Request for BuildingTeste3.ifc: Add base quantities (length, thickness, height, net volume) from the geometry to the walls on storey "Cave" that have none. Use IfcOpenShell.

First a look at what the model holds.

```python
import ifcopenshell
import ifcopenshell.util.element
import ifcopenshell.util.unit

model = ifcopenshell.open("BuildingTeste3.ifc")
print(model.schema)
for unit_type in ("LENGTHUNIT", "AREAUNIT", "VOLUMEUNIT"):
    print(unit_type, ifcopenshell.util.unit.calculate_unit_scale(model, unit_type))
storey = next(s for s in model.by_type("IfcBuildingStorey") if s.Name == "Cave")
walls = [e for e in ifcopenshell.util.element.get_decomposition(storey) if e.is_a("IfcWall")]
for e in sorted(walls, key=lambda e: e.id()):
    print(e.id(), e.is_a(), e.Name, list(ifcopenshell.util.element.get_psets(e, qtos_only=True)), sep=" | ")
```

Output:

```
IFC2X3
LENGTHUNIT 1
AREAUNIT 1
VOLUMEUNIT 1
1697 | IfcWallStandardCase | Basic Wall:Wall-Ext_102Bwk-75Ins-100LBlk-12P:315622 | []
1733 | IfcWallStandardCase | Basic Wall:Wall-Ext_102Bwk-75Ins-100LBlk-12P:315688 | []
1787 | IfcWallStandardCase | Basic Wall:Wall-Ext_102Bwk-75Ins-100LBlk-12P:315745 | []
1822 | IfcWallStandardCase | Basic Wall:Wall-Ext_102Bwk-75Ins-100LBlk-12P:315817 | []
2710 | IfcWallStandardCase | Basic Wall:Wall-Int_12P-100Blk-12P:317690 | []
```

```python
import ifcopenshell
import ifcopenshell.api.pset
import ifcopenshell.geom
import ifcopenshell.util.element
import ifcopenshell.util.shape
import ifcopenshell.util.unit

model = ifcopenshell.open("BuildingTeste3.ifc")
unit_scale = ifcopenshell.util.unit.calculate_unit_scale(model)
volume_scale = ifcopenshell.util.unit.calculate_unit_scale(model, "VOLUMEUNIT")
settings = ifcopenshell.geom.settings()

storey = next(s for s in model.by_type("IfcBuildingStorey") if s.Name == "Cave")
walls = [e for e in ifcopenshell.util.element.get_decomposition(storey) if e.is_a("IfcWall")]

for e in sorted(walls, key=lambda e: e.id()):
    if ifcopenshell.util.element.get_psets(e, qtos_only=True, should_inherit=False):
        continue
    # Geometry comes back in metres, in the element's own axes.
    shape = ifcopenshell.geom.create_shape(settings, e)
    values = {
        "Length": ifcopenshell.util.shape.get_x(shape.geometry) / unit_scale,
        "Width": ifcopenshell.util.shape.get_y(shape.geometry) / unit_scale,
        "Height": ifcopenshell.util.shape.get_z(shape.geometry) / unit_scale,
        "NetVolume": ifcopenshell.util.shape.get_volume(shape.geometry) / volume_scale,
    }
    qto = ifcopenshell.api.pset.add_qto(model, product=e, name="BaseQuantities")
    ifcopenshell.api.pset.edit_qto(model, qto=qto, properties=values)
    print(e.id(), {k: round(v, 3) for k, v in values.items()})

model.write("BuildingTeste3_rev.ifc")
```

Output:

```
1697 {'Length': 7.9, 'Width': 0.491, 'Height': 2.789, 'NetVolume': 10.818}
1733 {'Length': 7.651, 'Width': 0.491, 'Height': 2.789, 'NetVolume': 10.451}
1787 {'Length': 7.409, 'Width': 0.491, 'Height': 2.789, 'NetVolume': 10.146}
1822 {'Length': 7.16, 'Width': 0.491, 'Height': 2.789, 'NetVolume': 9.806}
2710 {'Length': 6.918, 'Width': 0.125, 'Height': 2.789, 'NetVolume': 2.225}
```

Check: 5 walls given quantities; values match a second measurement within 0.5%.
